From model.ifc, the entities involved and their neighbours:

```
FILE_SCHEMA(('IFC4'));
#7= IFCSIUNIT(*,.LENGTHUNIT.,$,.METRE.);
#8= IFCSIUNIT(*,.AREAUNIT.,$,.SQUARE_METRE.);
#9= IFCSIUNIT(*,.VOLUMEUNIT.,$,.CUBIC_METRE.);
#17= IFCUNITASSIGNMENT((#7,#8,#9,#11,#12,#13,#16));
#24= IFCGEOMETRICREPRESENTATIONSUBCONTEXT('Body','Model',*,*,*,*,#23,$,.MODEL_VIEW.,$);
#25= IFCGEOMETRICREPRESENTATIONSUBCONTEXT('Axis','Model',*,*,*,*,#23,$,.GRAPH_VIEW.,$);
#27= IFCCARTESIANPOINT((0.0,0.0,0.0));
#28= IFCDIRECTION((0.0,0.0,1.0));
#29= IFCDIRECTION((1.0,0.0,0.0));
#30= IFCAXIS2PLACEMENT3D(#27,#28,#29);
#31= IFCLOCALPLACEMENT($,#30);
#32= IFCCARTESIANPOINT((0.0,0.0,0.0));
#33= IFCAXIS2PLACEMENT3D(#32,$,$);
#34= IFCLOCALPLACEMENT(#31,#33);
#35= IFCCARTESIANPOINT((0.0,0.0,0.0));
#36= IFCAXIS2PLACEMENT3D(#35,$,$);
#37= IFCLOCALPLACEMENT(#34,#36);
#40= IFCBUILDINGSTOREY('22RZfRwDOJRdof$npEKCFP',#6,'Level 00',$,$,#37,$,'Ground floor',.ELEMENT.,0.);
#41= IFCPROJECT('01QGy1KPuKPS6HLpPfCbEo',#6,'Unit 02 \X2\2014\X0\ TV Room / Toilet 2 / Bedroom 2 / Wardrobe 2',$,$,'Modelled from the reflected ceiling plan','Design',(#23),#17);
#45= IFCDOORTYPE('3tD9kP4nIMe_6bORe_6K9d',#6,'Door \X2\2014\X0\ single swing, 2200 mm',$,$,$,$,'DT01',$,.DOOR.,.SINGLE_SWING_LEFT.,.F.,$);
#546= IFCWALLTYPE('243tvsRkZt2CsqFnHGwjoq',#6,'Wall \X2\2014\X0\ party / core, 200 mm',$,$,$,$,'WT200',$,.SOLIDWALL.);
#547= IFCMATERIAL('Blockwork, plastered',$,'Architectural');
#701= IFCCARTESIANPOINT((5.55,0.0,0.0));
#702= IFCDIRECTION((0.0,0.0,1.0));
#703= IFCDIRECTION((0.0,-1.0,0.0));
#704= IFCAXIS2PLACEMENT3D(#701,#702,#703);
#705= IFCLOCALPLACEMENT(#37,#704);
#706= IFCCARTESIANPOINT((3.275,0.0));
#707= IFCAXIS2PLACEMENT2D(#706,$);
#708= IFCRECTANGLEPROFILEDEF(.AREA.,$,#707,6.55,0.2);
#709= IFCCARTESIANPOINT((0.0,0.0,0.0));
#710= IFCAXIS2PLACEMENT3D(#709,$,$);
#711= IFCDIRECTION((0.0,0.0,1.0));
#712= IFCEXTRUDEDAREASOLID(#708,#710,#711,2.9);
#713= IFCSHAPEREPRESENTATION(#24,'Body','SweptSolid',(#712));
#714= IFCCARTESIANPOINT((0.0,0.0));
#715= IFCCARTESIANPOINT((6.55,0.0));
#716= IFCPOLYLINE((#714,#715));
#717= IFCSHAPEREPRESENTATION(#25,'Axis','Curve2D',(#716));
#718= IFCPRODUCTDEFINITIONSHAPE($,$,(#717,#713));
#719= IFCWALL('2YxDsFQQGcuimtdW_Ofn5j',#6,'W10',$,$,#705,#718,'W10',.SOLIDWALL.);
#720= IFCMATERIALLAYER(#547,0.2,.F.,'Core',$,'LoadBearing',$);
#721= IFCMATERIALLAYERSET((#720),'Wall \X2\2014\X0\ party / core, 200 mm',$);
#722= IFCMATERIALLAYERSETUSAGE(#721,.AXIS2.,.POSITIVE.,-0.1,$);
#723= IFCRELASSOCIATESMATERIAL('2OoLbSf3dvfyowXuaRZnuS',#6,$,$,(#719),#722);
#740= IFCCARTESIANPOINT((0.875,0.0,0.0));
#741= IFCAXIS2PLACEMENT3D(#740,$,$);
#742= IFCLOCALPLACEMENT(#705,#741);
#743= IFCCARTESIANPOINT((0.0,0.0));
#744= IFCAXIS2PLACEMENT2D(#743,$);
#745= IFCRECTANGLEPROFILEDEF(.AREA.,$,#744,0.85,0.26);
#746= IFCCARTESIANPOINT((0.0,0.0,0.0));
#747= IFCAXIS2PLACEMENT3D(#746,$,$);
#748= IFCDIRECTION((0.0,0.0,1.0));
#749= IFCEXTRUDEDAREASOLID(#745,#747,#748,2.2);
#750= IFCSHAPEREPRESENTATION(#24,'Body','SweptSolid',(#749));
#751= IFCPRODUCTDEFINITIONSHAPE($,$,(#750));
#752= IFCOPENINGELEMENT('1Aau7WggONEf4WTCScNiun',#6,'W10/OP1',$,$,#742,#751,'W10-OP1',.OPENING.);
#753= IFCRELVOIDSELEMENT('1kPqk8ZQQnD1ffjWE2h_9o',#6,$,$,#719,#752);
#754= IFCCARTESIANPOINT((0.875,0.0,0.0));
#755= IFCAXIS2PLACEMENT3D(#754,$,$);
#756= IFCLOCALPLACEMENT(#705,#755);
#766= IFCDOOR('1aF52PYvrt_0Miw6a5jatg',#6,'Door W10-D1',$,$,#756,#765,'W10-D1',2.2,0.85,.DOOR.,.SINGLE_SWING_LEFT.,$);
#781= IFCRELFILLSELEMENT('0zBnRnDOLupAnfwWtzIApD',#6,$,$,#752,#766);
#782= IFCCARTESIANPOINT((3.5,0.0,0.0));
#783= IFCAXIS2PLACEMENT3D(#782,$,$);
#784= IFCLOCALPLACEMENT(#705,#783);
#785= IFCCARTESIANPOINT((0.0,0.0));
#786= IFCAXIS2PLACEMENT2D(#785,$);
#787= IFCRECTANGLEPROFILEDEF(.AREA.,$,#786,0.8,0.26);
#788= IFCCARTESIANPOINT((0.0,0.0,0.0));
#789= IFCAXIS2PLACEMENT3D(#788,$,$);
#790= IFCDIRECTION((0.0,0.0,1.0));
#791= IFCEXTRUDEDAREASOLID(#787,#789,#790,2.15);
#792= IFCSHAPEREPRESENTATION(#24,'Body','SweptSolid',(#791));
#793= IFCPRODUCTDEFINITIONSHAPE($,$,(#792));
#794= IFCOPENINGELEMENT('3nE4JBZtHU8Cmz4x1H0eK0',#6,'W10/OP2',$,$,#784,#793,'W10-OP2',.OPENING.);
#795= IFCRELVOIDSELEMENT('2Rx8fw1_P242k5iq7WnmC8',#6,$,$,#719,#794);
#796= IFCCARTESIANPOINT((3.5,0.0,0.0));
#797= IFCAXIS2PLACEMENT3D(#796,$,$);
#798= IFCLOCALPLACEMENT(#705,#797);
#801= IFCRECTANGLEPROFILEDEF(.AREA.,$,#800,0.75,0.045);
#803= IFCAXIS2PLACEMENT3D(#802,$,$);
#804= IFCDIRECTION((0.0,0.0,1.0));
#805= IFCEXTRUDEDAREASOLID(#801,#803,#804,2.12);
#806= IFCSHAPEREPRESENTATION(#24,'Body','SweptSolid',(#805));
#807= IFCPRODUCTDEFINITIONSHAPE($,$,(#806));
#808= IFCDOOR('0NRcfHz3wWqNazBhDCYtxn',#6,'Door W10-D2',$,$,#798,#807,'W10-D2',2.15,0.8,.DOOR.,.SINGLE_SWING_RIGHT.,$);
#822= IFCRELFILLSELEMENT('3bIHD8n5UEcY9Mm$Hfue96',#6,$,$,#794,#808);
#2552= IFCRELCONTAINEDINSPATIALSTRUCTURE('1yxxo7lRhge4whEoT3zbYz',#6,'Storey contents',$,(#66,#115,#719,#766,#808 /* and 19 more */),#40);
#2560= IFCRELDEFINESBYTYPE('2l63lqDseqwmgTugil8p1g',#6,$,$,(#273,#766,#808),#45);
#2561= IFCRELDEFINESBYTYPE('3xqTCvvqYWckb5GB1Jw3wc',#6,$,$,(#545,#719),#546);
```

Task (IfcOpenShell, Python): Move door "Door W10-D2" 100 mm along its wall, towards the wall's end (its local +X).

```python
import ifcopenshell
import ifcopenshell.api.geometry
import ifcopenshell.util.placement

model = ifcopenshell.open("model.ifc")

door = model.by_guid("0NRcfHz3wWqNazBhDCYtxn")
opening = door.FillsVoids[0].RelatingOpeningElement
wall = opening.VoidsElements[0].RelatingBuildingElement

wall_matrix = ifcopenshell.util.placement.get_local_placement(wall.ObjectPlacement)
shift = wall_matrix[:3, 0] * 0.1
before = ifcopenshell.util.placement.get_local_placement(door.ObjectPlacement)[:3, 3].copy()

# The door is not placed relative to its opening, so move both.
for product in (opening, door):
    matrix = ifcopenshell.util.placement.get_local_placement(product.ObjectPlacement)
    matrix[:3, 3] += shift
    ifcopenshell.api.geometry.edit_object_placement(model, product=product, matrix=matrix, is_si=False)

after = ifcopenshell.util.placement.get_local_placement(door.ObjectPlacement)[:3, 3]
print("door moved by", (after - before).round(3) + 0.0)

model.write("model_updated.ifc")
```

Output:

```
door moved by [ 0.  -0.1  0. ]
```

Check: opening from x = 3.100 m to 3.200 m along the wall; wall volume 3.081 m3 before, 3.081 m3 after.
